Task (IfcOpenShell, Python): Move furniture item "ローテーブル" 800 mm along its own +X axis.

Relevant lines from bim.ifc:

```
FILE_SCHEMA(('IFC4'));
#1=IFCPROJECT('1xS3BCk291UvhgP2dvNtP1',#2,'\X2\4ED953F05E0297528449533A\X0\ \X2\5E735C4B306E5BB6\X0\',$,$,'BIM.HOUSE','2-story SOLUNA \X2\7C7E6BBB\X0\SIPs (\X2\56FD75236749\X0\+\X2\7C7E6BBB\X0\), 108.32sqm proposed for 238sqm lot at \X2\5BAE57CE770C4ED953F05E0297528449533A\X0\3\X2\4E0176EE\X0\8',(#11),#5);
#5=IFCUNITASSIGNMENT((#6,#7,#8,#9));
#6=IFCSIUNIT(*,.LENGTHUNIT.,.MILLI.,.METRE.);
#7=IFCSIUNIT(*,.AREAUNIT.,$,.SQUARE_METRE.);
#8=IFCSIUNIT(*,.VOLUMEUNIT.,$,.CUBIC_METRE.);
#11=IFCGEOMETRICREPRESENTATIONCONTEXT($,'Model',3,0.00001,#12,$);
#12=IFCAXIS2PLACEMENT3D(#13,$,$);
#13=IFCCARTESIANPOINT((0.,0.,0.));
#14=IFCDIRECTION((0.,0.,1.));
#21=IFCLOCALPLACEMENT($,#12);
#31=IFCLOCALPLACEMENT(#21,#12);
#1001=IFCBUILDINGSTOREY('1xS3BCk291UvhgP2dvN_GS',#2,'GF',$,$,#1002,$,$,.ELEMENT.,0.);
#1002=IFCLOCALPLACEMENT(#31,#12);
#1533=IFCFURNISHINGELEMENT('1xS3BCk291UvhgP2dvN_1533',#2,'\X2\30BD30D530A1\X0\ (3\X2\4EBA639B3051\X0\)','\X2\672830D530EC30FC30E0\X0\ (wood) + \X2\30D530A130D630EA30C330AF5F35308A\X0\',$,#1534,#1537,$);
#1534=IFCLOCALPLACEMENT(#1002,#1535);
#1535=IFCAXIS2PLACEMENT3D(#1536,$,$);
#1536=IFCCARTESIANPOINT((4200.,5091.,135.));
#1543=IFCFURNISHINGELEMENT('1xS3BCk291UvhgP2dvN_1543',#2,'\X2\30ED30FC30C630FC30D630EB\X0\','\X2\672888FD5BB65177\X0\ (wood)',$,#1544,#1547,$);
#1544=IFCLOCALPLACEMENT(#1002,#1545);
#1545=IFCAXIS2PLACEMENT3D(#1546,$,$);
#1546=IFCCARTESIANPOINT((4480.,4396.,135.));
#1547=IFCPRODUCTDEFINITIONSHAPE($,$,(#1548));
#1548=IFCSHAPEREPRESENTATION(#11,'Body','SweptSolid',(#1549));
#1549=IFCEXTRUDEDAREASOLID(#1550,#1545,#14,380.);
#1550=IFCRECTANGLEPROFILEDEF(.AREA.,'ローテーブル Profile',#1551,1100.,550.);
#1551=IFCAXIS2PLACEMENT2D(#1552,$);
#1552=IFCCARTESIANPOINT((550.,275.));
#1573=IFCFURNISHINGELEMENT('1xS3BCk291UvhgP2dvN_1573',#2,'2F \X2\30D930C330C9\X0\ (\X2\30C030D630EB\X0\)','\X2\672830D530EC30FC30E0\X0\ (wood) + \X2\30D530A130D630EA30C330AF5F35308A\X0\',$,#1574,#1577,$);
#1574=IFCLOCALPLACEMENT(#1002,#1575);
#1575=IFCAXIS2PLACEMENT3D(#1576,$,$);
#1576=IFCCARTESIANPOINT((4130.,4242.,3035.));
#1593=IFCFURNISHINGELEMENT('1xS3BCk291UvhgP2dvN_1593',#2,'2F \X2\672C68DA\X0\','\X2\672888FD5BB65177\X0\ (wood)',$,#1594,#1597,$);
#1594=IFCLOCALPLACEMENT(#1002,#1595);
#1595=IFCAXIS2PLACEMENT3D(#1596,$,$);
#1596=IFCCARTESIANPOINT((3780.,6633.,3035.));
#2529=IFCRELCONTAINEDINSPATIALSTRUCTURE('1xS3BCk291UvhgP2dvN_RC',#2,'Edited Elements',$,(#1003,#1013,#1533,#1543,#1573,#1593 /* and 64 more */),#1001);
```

```python
import ifcopenshell
import ifcopenshell.api.geometry
import ifcopenshell.util.placement
import ifcopenshell.util.unit

model = ifcopenshell.open("bim.ifc")
unit_scale = ifcopenshell.util.unit.calculate_unit_scale(model)

item = model.by_guid("1xS3BCk291UvhgP2dvN_1543")
matrix = ifcopenshell.util.placement.get_local_placement(item.ObjectPlacement)
matrix[:3, 3] += matrix[:3, 0] * 0.8 / unit_scale
ifcopenshell.api.geometry.edit_object_placement(model, product=item, matrix=matrix, is_si=False)

print(ifcopenshell.util.placement.get_local_placement(item.ObjectPlacement).round(3) + 0.0)

model.write("bim-out.ifc")
```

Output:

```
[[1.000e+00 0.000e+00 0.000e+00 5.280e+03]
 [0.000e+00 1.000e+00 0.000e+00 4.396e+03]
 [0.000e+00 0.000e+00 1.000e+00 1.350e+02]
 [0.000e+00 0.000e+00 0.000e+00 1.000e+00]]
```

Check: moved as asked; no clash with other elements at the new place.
